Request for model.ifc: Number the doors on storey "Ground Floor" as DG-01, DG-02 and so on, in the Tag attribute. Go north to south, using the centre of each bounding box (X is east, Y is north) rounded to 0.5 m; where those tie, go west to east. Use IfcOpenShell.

First a look at what the model holds.

```python
import ifcopenshell
import ifcopenshell.util.element
import ifcopenshell.util.placement

model = ifcopenshell.open("model.ifc")
print(model.schema)
storey = next(s for s in model.by_type("IfcBuildingStorey") if s.Name == "Ground Floor")
doors = [e for e in ifcopenshell.util.element.get_decomposition(storey) if e.is_a("IfcDoor")]
for e in sorted(doors, key=lambda e: e.id()):
    origin = ifcopenshell.util.placement.get_local_placement(e.ObjectPlacement)[:3, 3]
    print(e.id(), e.Tag, e.Name, origin.round(2) + 0.0, sep=" | ")
```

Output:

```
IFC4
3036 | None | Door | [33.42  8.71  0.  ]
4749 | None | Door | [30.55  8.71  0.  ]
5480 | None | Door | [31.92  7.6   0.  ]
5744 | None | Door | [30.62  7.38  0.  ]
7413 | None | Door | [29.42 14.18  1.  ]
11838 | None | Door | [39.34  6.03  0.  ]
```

```python
import ifcopenshell
import ifcopenshell.geom
import ifcopenshell.util.element
import ifcopenshell.util.shape

model = ifcopenshell.open("model.ifc")
settings = ifcopenshell.geom.settings()
settings.set("use-world-coords", True)


def centre(element):
    shape = ifcopenshell.geom.create_shape(settings, element)
    return ifcopenshell.util.shape.get_bbox_centroid(shape.geometry)


storey = next(s for s in model.by_type("IfcBuildingStorey") if s.Name == "Ground Floor")
doors = [e for e in ifcopenshell.util.element.get_decomposition(storey) if e.is_a("IfcDoor")]

# Insertion points can sit at a corner or the storey origin, so sort by the geometry (in metres).
centres = {e: centre(e) for e in doors}
doors.sort(key=lambda e: (-round(centres[e][1] / 0.5), centres[e][0]))

for i, e in enumerate(doors, start=1):
    number = f"DG-{i:02d}"
    e.Tag = number
    print(e.id(), number)

model.write("model_edited.ifc")
```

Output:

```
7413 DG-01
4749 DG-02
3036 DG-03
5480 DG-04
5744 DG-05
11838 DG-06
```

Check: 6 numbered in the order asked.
